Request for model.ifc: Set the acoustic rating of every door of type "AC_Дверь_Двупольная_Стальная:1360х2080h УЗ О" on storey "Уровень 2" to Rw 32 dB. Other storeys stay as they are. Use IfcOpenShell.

First a look at what the model holds.

```python
import ifcopenshell
import ifcopenshell.util.element

model = ifcopenshell.open("model.ifc")
print(model.schema)
storey = next(s for s in model.by_type("IfcBuildingStorey") if s.Name == "Уровень 2")
doors = [e for e in ifcopenshell.util.element.get_decomposition(storey) if e.is_a("IfcDoor")]
seen = {}
for e in doors:
    element_type = ifcopenshell.util.element.get_type(e)
    key = (element_type.Name if element_type != e and element_type else None, ifcopenshell.util.element.get_pset(e, "Pset_DoorCommon", "AcousticRating"))
    seen[key] = seen.get(key, 0) + 1
for (name, value), count in sorted(seen.items(), key=str):
    print(count, "x", name, "|", value)
```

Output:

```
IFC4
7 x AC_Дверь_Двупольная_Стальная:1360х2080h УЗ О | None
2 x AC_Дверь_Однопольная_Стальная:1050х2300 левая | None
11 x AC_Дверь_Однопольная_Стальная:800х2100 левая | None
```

```python
import ifcopenshell
import ifcopenshell.api.pset
import ifcopenshell.util.element

model = ifcopenshell.open("model.ifc")

storey = next(s for s in model.by_type("IfcBuildingStorey") if s.Name == "Уровень 2")
doors = [e for e in ifcopenshell.util.element.get_decomposition(storey) if e.is_a("IfcDoor")]

count = 0
for e in doors:
    element_type = ifcopenshell.util.element.get_type(e)
    if element_type in (None, e) or element_type.Name != "AC_Дверь_Двупольная_Стальная:1360х2080h УЗ О":
        continue
    # add_pset returns the element's existing set when there is one.
    pset = ifcopenshell.api.pset.add_pset(model, product=e, name="Pset_DoorCommon")
    ifcopenshell.api.pset.edit_pset(model, pset=pset, properties={"AcousticRating": "Rw 32 dB"})
    count += 1

print(count, "doors updated")

model.write("model_edited.ifc")
```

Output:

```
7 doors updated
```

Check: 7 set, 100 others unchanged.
